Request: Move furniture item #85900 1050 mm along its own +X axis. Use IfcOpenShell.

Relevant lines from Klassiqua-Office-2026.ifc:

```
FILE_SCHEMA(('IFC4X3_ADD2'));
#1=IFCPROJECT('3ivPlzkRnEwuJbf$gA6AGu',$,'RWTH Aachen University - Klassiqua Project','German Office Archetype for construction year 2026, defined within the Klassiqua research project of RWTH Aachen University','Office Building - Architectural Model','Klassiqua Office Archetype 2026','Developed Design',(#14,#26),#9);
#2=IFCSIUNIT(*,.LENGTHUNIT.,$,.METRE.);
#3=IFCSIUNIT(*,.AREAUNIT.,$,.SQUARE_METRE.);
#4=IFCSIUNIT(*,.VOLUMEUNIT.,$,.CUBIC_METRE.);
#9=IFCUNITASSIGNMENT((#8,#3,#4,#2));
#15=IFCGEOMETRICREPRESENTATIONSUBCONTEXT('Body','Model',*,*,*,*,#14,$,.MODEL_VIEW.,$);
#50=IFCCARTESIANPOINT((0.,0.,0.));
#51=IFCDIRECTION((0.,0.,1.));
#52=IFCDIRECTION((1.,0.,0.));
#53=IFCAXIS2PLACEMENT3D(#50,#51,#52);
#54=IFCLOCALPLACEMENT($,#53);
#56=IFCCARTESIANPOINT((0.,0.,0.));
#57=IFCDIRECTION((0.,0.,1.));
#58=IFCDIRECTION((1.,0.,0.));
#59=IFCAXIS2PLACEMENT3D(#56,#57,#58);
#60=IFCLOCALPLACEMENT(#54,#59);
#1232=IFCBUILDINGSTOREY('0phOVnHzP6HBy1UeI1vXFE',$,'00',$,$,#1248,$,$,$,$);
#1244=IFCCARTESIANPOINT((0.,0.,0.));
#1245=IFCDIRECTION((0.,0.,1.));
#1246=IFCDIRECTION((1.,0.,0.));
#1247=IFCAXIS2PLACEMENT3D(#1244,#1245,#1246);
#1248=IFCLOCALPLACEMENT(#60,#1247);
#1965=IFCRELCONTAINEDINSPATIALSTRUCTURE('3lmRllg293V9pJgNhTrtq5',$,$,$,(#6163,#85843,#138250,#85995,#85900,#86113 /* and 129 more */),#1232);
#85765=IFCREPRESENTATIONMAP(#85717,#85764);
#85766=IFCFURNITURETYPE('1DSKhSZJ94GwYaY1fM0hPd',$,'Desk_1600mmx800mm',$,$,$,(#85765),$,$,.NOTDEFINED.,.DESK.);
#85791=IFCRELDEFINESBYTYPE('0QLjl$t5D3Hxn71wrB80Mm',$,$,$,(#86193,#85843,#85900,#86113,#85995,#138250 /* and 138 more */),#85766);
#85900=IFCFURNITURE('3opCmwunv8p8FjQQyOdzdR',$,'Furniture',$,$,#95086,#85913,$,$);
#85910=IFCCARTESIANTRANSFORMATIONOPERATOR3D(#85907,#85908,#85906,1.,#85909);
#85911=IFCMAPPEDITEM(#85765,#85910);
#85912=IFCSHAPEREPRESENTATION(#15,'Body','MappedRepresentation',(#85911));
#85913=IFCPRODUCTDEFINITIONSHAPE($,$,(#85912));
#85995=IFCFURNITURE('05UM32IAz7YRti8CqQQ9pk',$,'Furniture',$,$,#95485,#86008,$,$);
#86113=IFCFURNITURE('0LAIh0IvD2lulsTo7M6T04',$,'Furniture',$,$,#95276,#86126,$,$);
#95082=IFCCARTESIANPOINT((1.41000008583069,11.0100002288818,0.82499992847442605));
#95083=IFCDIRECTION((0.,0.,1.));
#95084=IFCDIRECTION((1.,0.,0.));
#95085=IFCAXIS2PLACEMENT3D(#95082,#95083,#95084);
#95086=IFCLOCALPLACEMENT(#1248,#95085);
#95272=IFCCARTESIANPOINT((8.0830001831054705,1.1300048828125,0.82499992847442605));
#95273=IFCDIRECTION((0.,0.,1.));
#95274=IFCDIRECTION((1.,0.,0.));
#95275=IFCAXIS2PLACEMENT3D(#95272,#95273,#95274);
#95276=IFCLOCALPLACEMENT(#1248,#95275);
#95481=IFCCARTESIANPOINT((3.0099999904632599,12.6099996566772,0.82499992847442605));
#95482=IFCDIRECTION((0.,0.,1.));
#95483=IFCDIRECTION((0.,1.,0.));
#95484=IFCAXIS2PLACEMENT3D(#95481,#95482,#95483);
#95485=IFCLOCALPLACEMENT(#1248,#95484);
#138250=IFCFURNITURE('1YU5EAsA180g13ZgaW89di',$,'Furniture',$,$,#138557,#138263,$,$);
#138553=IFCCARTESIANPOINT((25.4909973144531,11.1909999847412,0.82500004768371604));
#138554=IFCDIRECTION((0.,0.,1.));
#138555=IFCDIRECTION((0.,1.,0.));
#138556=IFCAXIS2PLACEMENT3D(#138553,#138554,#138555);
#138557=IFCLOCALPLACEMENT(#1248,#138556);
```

```python
import ifcopenshell
import ifcopenshell.api.geometry
import ifcopenshell.util.placement

model = ifcopenshell.open("Klassiqua-Office-2026.ifc")

item = model.by_id(85900)
matrix = ifcopenshell.util.placement.get_local_placement(item.ObjectPlacement)
matrix[:3, 3] += matrix[:3, 0] * 1.05
ifcopenshell.api.geometry.edit_object_placement(model, product=item, matrix=matrix, is_si=False)

print(ifcopenshell.util.placement.get_local_placement(item.ObjectPlacement).round(3) + 0.0)

model.write("Klassiqua-Office-2026-out.ifc")
```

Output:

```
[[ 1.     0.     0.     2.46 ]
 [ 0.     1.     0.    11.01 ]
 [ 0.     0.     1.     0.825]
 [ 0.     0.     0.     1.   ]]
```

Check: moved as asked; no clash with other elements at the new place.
